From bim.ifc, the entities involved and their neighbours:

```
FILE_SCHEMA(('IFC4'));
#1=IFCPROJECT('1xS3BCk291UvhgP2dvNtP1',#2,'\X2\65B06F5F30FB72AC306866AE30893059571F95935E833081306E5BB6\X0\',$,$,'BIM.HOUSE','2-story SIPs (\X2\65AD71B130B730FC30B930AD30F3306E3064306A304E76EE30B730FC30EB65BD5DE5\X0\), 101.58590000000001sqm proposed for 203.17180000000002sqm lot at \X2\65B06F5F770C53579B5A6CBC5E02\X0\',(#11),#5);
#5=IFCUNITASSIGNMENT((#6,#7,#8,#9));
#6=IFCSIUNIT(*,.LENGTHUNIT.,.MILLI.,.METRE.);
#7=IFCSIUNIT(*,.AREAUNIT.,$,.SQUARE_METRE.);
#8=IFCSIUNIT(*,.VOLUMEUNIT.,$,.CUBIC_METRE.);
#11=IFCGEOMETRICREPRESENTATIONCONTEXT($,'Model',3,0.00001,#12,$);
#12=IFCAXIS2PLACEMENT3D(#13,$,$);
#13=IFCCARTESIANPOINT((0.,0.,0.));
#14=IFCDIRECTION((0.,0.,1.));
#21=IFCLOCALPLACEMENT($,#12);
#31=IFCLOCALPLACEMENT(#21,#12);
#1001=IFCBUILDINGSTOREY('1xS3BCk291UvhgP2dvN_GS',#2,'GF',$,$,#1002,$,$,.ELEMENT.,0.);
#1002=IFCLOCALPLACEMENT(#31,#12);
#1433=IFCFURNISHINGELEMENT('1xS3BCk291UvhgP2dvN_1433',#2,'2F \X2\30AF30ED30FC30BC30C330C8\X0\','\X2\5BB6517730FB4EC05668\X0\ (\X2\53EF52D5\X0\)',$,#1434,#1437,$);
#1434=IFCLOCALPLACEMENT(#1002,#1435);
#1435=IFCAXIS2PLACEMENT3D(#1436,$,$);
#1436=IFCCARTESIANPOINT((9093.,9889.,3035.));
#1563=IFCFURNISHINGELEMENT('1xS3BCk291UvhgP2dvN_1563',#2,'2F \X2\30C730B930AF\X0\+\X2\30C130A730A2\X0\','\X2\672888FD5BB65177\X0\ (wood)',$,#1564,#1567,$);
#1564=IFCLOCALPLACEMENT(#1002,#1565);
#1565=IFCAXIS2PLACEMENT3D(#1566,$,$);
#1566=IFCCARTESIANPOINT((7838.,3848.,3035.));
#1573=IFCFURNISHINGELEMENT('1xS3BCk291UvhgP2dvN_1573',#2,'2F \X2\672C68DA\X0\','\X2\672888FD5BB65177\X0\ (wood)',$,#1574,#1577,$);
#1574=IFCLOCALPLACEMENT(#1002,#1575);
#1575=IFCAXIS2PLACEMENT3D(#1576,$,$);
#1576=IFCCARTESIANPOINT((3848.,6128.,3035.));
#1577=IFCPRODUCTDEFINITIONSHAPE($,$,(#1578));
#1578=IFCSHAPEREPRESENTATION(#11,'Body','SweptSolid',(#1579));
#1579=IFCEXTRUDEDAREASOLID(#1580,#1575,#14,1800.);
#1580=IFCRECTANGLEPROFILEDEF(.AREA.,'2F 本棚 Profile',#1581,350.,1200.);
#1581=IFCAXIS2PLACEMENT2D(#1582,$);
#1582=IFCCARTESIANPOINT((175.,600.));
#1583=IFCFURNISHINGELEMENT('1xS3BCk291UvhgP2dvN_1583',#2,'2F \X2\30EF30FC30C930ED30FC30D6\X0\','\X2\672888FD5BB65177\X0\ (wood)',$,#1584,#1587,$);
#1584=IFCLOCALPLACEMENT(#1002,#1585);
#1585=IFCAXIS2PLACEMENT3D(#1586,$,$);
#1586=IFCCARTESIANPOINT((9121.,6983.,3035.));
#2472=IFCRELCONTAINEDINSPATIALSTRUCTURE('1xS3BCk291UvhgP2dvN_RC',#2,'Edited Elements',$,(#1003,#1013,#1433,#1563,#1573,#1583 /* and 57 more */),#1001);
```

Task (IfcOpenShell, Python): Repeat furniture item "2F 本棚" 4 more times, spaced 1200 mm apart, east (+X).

```python
import numpy as np
import ifcopenshell
import ifcopenshell.api.geometry
import ifcopenshell.api.root
import ifcopenshell.util.element
import ifcopenshell.util.placement
import ifcopenshell.util.unit

model = ifcopenshell.open("bim.ifc")
unit_scale = ifcopenshell.util.unit.calculate_unit_scale(model)


def reuse_history(source, copy):
    """copy_class also copies each property set's owner history, people and application; keep the originals."""
    for rel in copy.IsDefinedBy:
        if rel.is_a("IfcRelDefinesByProperties") and (history := rel.RelatingPropertyDefinition.OwnerHistory):
            rel.RelatingPropertyDefinition.OwnerHistory = source.OwnerHistory
            ifcopenshell.util.element.remove_deep2(model, history)


source = model.by_guid("1xS3BCk291UvhgP2dvN_1573")
base = ifcopenshell.util.placement.get_local_placement(source.ObjectPlacement)
step = np.array([1.0, 0.0, 0.0]) * 1.2 / unit_scale

for i in range(1, 5):
    copy = ifcopenshell.api.root.copy_class(model, product=source)
    copy.Representation = ifcopenshell.util.element.copy_deep(
        model, source.Representation, exclude=["IfcGeometricRepresentationContext", "IfcRepresentationMap"]
    )
    reuse_history(source, copy)
    matrix = base.copy()
    matrix[:3, 3] += i * step
    print("added at", matrix[:3, 3].round(3) + 0.0)
    ifcopenshell.api.geometry.edit_object_placement(model, product=copy, matrix=matrix, is_si=False)

model.write("bim-out.ifc")
```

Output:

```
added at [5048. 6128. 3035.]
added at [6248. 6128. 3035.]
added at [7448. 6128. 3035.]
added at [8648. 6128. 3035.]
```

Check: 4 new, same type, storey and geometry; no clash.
